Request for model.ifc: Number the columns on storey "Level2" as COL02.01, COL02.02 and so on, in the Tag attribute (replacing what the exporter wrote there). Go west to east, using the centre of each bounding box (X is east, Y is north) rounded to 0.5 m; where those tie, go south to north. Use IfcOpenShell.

First a look at what the model holds.

```python
import ifcopenshell
import ifcopenshell.util.element
import ifcopenshell.util.placement

model = ifcopenshell.open("model.ifc")
print(model.schema)
storey = next(s for s in model.by_type("IfcBuildingStorey") if s.Name == "Level2")
columns = [e for e in ifcopenshell.util.element.get_decomposition(storey) if e.is_a("IfcColumn")]
for e in sorted(columns, key=lambda e: e.id()):
    origin = ifcopenshell.util.placement.get_local_placement(e.ObjectPlacement)[:3, 3]
    print(e.id(), e.Tag, e.Name, origin.round(2) + 0.0, sep=" | ")
```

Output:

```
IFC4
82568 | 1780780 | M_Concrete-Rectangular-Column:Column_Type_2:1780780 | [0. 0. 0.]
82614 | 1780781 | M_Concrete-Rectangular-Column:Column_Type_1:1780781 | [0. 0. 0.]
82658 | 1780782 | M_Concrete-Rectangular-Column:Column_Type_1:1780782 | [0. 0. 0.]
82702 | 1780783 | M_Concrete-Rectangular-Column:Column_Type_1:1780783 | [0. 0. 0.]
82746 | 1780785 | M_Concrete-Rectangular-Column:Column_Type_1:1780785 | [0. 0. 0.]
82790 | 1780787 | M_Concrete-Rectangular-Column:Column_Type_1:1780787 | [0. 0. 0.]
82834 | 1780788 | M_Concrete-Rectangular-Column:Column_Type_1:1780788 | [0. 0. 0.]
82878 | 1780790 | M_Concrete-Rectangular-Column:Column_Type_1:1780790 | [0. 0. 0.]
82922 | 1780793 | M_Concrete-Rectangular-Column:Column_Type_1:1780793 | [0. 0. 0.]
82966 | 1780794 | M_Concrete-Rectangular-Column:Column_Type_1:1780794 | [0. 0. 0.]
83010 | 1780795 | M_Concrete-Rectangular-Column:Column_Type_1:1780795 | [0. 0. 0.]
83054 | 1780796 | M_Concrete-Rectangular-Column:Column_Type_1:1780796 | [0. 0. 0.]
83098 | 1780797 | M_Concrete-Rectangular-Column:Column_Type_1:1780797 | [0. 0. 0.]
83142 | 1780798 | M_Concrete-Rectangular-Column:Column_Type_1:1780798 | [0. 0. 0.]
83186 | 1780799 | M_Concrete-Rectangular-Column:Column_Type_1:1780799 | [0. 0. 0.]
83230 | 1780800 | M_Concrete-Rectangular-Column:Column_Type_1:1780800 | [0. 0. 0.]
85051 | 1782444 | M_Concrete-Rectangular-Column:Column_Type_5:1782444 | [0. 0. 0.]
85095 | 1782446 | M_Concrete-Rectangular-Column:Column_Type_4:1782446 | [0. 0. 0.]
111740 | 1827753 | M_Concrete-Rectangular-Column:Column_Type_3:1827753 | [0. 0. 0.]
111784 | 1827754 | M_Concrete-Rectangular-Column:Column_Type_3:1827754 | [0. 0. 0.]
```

```python
import ifcopenshell
import ifcopenshell.geom
import ifcopenshell.util.element
import ifcopenshell.util.shape

model = ifcopenshell.open("model.ifc")
settings = ifcopenshell.geom.settings()
settings.set("use-world-coords", True)


def centre(element):
    shape = ifcopenshell.geom.create_shape(settings, element)
    return ifcopenshell.util.shape.get_bbox_centroid(shape.geometry)


storey = next(s for s in model.by_type("IfcBuildingStorey") if s.Name == "Level2")
columns = [e for e in ifcopenshell.util.element.get_decomposition(storey) if e.is_a("IfcColumn")]

# Insertion points can sit at a corner or the storey origin, so sort by the geometry (in metres).
centres = {e: centre(e) for e in columns}
columns.sort(key=lambda e: (round(centres[e][0] / 0.5), centres[e][1]))

for i, e in enumerate(columns, start=1):
    number = f"COL02.{i:02d}"
    e.Tag = number
    print(e.id(), number)

model.write("model-out.ifc")
```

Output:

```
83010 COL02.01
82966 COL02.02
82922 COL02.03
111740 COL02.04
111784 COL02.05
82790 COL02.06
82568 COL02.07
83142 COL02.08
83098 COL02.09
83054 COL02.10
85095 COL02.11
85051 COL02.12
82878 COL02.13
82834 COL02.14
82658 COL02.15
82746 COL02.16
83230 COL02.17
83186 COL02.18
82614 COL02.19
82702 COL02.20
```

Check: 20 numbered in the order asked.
